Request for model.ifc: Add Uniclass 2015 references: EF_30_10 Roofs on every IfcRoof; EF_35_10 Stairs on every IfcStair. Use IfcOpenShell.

First a look at what the model holds.

```python
import ifcopenshell

model = ifcopenshell.open("model.ifc")
print(model.schema)
print("classifications:", [c.Name for c in model.by_type("IfcClassification")])
for ifc_class in ("IfcDoor", "IfcRoof", "IfcStair", "IfcWall", "IfcWindow"):
    print(ifc_class, len(model.by_type(ifc_class)))
```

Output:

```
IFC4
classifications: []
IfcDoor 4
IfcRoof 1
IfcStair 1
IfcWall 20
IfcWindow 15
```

```python
import ifcopenshell
import ifcopenshell.api.classification

model = ifcopenshell.open("model.ifc")

system = ifcopenshell.api.classification.add_classification(model, classification="Uniclass 2015")

codes = {
    "IfcRoof": ("EF_30_10", "Roofs"),
    "IfcStair": ("EF_35_10", "Stairs"),
}
for ifc_class, (code, name) in codes.items():
    products = model.by_type(ifc_class)
    ifcopenshell.api.classification.add_reference(
        model, products=products, classification=system, identification=code, name=name
    )
    print(code, len(products))

model.write("model_updated.ifc")
```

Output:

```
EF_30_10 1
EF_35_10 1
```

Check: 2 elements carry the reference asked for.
